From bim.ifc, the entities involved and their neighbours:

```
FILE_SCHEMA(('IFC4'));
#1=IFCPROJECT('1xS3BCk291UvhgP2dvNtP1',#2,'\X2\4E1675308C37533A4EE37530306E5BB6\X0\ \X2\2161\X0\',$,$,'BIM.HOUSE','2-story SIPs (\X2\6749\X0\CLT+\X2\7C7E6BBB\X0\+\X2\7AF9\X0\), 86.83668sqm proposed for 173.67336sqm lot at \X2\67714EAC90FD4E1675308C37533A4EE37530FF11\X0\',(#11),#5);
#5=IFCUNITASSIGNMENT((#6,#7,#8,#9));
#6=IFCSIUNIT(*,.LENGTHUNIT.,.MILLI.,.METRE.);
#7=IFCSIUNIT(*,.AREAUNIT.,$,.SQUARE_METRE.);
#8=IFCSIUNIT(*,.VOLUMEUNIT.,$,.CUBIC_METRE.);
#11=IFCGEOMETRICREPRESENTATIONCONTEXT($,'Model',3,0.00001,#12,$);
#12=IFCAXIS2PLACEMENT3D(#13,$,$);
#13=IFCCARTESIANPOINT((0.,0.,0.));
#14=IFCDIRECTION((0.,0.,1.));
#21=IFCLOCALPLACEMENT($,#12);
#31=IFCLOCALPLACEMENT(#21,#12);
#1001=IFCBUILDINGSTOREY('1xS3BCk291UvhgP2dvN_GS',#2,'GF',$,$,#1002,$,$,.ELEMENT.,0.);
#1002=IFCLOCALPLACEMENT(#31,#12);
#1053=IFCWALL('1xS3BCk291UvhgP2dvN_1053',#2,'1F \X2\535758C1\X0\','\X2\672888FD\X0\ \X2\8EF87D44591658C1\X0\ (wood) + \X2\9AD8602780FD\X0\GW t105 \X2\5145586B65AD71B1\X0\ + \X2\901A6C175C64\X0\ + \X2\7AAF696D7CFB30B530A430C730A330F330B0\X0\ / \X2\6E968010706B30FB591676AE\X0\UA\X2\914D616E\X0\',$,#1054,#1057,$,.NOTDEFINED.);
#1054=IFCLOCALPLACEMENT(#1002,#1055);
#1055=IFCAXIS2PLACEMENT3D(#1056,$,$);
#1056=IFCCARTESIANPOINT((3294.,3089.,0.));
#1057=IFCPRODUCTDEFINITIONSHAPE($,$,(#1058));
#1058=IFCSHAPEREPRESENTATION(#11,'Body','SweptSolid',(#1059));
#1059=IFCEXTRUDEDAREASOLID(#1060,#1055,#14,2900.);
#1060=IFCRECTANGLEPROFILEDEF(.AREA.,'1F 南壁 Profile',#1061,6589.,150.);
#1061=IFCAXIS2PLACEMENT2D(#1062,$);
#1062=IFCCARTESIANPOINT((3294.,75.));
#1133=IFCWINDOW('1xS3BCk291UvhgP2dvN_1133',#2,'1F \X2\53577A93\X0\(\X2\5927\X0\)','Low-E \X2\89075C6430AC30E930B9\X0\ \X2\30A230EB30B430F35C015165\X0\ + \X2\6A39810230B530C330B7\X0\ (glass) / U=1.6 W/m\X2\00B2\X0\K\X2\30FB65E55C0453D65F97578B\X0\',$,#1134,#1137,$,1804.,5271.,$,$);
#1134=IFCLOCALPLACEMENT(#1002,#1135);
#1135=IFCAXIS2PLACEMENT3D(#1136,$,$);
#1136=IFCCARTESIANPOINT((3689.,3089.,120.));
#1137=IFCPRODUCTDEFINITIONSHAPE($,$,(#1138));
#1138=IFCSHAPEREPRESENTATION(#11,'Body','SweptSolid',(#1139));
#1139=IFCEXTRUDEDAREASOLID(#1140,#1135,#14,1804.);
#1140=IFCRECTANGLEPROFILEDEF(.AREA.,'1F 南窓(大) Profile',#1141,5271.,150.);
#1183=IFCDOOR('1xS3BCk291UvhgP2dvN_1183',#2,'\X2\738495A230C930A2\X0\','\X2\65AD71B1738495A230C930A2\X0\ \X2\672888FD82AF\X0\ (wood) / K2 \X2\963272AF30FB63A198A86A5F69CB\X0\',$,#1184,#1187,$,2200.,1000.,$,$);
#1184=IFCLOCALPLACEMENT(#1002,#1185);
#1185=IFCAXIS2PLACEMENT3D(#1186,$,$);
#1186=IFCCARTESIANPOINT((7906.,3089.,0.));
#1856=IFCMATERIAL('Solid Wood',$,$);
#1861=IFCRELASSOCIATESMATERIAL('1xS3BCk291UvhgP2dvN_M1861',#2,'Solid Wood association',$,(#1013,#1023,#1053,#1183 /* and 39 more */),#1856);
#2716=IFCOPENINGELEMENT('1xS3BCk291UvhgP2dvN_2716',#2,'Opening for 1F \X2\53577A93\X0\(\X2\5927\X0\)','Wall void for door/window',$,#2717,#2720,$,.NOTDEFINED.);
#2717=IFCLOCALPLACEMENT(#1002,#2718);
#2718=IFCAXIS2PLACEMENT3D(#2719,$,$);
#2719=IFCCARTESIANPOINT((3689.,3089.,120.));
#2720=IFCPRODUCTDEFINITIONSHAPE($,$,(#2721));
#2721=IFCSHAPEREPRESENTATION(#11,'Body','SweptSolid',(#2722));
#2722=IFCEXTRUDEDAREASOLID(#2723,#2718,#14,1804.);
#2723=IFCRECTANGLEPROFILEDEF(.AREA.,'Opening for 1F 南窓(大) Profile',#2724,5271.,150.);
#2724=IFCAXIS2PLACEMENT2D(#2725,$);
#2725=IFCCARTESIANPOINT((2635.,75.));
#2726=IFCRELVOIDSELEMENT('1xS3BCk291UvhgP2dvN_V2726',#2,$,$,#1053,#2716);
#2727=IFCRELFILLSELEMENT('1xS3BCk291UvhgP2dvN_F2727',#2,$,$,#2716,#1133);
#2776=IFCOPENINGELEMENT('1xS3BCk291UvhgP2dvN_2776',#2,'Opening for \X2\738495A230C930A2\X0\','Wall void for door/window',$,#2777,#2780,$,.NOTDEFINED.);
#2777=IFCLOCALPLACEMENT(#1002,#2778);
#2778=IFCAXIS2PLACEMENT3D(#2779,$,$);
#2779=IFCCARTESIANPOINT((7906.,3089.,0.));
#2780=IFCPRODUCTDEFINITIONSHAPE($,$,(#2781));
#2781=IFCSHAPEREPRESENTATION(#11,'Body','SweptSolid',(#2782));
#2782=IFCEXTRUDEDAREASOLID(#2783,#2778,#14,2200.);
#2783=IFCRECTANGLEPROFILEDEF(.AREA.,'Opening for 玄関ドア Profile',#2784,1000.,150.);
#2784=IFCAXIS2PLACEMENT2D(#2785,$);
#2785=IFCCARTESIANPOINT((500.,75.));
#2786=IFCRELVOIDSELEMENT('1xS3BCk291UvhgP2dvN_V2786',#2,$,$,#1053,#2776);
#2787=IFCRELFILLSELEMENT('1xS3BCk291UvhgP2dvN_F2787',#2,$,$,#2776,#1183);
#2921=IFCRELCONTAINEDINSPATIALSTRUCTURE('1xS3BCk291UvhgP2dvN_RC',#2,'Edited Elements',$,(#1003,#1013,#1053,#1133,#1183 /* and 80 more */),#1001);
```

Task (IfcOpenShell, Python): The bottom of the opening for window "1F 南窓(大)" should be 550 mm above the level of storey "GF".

```python
import numpy as np
import ifcopenshell
import ifcopenshell.api.geometry
import ifcopenshell.geom
import ifcopenshell.util.element
import ifcopenshell.util.placement
import ifcopenshell.util.shape
import ifcopenshell.util.unit

model = ifcopenshell.open("bim.ifc")
unit_scale = ifcopenshell.util.unit.calculate_unit_scale(model)

window = model.by_id(1133)
opening = window.FillsVoids[0].RelatingOpeningElement
storey = ifcopenshell.util.element.get_container(window, ifc_class="IfcBuildingStorey")
level = ifcopenshell.util.placement.get_local_placement(storey.ObjectPlacement)[2, 3]

# The opening's origin need not be at the sill, so measure its lowest point.
shape = ifcopenshell.geom.create_shape(ifcopenshell.geom.settings(), opening)
bottom = ifcopenshell.util.shape.get_shape_bottom_elevation(shape, shape.geometry) / unit_scale
dz = level + 550.0 - bottom

shift = np.array([0.0, 0.0, dz])
# The window is not placed relative to its opening, so move both.
for product in (opening, window):
    matrix = ifcopenshell.util.placement.get_local_placement(product.ObjectPlacement)
    matrix[:3, 3] += shift
    ifcopenshell.api.geometry.edit_object_placement(model, product=product, matrix=matrix, is_si=False)

print(f"moved by {dz * unit_scale:+.3f} m")

model.write("bim_rev.ifc")
```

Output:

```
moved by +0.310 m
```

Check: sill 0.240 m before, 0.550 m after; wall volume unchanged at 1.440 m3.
